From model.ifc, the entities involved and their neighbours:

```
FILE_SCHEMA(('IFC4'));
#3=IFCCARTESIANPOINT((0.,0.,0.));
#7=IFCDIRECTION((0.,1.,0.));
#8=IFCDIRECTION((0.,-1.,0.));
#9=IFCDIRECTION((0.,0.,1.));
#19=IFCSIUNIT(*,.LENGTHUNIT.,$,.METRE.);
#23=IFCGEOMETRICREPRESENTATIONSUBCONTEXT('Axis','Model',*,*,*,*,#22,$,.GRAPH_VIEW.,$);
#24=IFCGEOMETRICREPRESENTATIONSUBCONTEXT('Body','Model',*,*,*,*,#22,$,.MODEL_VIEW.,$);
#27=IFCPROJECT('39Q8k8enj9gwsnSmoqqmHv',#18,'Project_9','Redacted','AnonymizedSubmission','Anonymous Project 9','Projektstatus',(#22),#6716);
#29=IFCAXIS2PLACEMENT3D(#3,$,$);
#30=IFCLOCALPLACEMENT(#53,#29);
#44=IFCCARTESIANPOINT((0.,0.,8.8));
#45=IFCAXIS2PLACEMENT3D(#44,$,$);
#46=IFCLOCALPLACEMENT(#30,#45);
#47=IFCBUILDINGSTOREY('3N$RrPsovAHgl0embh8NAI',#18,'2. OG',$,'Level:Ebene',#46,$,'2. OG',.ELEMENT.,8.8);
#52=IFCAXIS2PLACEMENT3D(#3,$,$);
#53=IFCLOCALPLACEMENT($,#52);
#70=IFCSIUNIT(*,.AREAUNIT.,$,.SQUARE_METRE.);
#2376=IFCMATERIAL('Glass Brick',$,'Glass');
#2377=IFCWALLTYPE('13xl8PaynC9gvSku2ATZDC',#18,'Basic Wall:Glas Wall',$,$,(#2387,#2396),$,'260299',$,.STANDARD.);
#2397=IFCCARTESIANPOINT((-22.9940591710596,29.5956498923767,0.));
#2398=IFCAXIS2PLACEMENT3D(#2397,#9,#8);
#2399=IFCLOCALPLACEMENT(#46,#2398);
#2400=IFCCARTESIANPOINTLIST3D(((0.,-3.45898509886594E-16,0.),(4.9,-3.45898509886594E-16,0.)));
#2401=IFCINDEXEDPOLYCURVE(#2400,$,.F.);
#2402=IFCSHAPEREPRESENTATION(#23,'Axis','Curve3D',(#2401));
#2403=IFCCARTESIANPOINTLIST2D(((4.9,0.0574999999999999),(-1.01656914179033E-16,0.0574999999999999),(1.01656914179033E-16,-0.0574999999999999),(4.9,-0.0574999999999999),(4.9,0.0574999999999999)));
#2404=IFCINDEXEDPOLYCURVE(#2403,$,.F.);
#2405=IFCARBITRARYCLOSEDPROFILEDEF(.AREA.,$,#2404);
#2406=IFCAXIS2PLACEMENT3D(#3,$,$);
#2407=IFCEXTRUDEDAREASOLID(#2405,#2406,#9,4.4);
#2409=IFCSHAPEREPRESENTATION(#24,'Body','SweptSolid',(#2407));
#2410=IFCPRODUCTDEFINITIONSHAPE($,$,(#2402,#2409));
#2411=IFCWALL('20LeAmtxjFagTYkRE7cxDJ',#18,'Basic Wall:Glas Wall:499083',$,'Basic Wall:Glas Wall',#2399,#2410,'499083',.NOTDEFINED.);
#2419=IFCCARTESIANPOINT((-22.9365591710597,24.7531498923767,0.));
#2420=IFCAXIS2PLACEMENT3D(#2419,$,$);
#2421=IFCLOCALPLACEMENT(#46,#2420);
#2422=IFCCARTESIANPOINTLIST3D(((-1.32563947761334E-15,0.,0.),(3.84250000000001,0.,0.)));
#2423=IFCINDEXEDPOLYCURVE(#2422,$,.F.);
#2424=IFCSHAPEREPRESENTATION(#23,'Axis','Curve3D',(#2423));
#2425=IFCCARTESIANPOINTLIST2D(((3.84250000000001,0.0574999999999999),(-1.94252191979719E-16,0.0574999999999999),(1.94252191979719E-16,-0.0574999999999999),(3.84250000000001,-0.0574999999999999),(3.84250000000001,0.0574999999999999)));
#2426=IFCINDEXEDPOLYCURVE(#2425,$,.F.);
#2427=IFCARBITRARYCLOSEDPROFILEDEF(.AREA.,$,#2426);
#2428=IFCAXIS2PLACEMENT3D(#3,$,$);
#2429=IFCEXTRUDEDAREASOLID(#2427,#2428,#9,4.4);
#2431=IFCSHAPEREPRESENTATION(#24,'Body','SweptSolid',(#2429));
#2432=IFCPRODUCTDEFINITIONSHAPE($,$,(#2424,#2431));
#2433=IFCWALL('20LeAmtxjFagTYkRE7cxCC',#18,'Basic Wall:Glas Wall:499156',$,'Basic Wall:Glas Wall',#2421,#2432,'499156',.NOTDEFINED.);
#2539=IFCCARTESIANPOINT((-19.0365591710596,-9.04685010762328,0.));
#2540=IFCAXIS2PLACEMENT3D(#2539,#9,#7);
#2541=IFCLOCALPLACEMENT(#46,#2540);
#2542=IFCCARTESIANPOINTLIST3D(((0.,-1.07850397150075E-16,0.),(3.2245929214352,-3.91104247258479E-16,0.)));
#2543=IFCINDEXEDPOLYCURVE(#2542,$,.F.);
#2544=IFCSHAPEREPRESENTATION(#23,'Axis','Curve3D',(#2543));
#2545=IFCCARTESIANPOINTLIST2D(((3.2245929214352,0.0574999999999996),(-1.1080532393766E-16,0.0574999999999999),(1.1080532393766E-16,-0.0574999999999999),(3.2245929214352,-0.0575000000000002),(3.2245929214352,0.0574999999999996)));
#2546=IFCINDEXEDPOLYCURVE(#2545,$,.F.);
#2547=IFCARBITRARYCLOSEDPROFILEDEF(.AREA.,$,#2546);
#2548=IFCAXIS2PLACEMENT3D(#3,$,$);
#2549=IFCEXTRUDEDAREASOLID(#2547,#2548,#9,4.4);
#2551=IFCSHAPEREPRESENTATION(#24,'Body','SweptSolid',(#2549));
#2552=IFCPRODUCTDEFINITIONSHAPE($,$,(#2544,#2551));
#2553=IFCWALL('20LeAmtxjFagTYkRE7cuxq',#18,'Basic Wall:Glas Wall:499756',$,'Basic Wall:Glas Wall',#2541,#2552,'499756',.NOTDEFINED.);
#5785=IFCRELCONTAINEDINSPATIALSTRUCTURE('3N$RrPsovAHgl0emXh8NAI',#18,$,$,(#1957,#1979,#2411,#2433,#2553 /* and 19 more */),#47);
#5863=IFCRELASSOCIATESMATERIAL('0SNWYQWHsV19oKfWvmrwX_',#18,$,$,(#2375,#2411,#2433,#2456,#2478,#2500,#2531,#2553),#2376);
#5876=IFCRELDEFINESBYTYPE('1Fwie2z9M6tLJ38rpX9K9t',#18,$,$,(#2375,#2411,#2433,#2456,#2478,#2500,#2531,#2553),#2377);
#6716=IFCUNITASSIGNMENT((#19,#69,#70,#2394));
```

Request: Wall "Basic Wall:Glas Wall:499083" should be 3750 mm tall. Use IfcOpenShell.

```python
import ifcopenshell
import ifcopenshell.geom
import ifcopenshell.util.representation
import ifcopenshell.util.shape

model = ifcopenshell.open("model.ifc")
settings = ifcopenshell.geom.settings()


def volume(element):
    """Net volume in cubic metres, openings subtracted."""
    shape = ifcopenshell.geom.create_shape(settings, element)
    return ifcopenshell.util.shape.get_volume(shape.geometry)


wall = model.by_guid("20LeAmtxjFagTYkRE7cxDJ")
before = volume(wall)

body = ifcopenshell.util.representation.get_representation(wall, "Model", "Body")
solid = body.Items[0]
old_height = solid.Depth
solid.Depth = 3.75
after = volume(wall)

print(f"height {old_height:g} -> {solid.Depth:g}, volume {before:.3f} -> {after:.3f} m3")

model.write("model_v2.ifc")
```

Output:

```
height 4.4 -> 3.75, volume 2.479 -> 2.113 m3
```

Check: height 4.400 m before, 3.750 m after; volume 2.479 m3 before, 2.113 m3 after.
